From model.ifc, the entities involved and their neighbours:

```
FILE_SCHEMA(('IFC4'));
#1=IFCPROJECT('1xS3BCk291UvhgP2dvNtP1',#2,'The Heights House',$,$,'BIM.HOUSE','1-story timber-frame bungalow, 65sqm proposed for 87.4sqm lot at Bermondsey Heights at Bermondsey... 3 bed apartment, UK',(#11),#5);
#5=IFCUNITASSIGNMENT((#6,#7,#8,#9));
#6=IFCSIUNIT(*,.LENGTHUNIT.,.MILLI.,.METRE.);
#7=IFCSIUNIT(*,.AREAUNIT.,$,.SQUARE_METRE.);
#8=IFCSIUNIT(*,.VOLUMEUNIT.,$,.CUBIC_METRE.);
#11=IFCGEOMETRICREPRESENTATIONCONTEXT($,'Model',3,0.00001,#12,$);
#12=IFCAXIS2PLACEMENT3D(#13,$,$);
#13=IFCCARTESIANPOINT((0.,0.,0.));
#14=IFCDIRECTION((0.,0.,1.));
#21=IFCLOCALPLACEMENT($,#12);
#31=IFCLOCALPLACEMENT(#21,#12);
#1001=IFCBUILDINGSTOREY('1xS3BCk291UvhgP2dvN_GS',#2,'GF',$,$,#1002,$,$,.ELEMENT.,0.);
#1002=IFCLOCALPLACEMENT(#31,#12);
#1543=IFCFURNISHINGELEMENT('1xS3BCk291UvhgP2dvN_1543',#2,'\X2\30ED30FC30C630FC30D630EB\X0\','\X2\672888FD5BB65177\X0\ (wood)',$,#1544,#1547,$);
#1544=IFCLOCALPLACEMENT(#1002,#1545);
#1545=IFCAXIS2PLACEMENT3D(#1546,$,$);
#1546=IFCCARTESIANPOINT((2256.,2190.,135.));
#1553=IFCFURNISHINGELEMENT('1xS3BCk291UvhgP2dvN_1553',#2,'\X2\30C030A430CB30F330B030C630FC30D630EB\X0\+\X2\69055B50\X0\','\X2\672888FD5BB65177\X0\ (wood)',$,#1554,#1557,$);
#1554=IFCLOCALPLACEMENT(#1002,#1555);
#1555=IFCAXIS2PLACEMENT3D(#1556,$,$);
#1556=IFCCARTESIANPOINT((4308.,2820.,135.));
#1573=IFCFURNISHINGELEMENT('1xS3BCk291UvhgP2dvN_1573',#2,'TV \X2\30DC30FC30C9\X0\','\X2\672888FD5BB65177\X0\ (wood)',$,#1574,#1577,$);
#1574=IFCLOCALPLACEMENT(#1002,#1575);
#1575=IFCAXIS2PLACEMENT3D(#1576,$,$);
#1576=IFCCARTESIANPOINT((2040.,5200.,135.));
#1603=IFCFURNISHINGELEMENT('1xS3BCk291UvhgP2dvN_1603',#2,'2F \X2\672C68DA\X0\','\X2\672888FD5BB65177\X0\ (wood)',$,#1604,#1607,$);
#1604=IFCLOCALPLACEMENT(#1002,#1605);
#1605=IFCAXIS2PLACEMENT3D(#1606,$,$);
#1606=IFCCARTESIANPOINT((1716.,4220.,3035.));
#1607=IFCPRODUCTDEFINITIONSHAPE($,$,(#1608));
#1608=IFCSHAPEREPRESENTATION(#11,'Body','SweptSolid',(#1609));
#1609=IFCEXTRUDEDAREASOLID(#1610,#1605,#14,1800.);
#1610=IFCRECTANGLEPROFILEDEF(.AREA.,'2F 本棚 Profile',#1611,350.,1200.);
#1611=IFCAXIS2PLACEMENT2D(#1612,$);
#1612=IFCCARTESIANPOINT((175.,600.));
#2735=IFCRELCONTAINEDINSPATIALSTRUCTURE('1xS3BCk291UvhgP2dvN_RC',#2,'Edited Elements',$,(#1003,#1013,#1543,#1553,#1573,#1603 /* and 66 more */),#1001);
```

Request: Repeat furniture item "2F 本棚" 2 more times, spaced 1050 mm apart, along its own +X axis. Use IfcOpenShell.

```python
import ifcopenshell
import ifcopenshell.api.geometry
import ifcopenshell.api.root
import ifcopenshell.util.element
import ifcopenshell.util.placement

model = ifcopenshell.open("model.ifc")


def reuse_history(source, copy):
    """copy_class also copies each property set's owner history, people and application; keep the originals."""
    for rel in copy.IsDefinedBy:
        if rel.is_a("IfcRelDefinesByProperties") and (history := rel.RelatingPropertyDefinition.OwnerHistory):
            rel.RelatingPropertyDefinition.OwnerHistory = source.OwnerHistory
            ifcopenshell.util.element.remove_deep2(model, history)


source = model.by_guid("1xS3BCk291UvhgP2dvN_1603")
base = ifcopenshell.util.placement.get_local_placement(source.ObjectPlacement)
step = base[:3, 0] * 1050.0

for i in range(1, 3):
    copy = ifcopenshell.api.root.copy_class(model, product=source)
    copy.Representation = ifcopenshell.util.element.copy_deep(
        model, source.Representation, exclude=["IfcGeometricRepresentationContext", "IfcRepresentationMap"]
    )
    reuse_history(source, copy)
    matrix = base.copy()
    matrix[:3, 3] += i * step
    print("added at", matrix[:3, 3].round(3) + 0.0)
    ifcopenshell.api.geometry.edit_object_placement(model, product=copy, matrix=matrix, is_si=False)

model.write("model_updated.ifc")
```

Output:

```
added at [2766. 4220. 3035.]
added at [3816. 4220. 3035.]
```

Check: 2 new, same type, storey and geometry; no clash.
